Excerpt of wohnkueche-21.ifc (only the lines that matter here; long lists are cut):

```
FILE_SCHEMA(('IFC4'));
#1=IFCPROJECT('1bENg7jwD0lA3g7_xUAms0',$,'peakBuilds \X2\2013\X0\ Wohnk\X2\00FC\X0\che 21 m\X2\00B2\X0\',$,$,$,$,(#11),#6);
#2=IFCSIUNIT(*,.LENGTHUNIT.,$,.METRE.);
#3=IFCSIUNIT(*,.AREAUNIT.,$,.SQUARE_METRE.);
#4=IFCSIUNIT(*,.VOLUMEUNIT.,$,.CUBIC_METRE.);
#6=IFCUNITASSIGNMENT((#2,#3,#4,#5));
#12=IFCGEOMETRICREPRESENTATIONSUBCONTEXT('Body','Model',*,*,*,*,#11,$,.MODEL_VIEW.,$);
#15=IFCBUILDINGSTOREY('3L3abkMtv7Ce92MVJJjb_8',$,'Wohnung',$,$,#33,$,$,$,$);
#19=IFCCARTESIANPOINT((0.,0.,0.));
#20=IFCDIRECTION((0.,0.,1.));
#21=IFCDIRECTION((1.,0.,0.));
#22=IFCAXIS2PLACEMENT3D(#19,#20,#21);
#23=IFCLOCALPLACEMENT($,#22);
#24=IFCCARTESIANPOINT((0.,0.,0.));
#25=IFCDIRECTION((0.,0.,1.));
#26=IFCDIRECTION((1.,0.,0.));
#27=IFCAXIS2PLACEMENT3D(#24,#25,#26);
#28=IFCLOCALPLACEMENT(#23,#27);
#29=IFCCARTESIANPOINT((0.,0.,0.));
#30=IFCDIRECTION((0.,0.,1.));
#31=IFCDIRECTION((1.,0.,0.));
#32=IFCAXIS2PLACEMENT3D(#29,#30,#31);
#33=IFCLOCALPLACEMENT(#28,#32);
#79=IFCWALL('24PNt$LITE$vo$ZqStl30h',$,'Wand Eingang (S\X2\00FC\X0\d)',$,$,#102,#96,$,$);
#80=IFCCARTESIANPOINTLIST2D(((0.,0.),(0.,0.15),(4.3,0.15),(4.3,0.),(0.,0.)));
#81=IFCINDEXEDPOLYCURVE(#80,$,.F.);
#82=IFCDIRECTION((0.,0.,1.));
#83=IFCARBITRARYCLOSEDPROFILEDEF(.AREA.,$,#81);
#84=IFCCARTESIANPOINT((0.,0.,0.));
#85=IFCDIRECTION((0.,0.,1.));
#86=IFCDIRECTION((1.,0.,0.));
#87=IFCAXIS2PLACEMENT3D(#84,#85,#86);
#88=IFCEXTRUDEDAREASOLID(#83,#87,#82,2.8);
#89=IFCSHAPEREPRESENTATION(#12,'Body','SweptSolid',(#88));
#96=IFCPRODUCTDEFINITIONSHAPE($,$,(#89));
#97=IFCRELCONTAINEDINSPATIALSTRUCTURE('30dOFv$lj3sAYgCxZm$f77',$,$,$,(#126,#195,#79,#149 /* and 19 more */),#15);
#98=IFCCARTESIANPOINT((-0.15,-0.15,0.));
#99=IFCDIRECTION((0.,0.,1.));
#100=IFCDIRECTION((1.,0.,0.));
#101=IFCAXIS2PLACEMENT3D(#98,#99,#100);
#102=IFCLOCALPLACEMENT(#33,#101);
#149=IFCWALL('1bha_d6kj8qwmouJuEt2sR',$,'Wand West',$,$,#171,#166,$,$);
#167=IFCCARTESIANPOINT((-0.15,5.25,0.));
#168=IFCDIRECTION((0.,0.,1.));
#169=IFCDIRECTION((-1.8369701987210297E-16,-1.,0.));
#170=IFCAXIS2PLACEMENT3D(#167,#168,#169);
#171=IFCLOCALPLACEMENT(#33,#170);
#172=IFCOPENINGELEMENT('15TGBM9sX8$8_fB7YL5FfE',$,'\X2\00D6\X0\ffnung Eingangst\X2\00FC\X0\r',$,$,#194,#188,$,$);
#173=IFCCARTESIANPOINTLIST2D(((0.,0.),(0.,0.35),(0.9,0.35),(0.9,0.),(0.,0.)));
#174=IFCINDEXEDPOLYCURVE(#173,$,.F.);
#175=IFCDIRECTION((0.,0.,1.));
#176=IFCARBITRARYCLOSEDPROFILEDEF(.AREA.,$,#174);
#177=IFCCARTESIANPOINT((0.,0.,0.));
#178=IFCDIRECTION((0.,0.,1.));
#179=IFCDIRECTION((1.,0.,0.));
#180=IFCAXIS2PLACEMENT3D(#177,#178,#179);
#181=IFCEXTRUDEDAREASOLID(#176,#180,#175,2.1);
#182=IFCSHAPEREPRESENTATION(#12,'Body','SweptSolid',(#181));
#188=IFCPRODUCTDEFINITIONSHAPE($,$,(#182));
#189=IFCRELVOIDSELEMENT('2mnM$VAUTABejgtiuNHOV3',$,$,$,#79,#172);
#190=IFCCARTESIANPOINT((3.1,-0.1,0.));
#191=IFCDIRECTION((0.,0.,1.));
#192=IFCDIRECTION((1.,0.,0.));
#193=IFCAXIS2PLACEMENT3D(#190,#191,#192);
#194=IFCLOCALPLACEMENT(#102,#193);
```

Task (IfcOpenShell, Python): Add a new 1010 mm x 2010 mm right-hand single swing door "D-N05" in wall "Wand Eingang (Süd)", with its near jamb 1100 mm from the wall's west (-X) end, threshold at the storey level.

```python
import numpy as np
import ifcopenshell
import ifcopenshell.api.feature
import ifcopenshell.api.geometry
import ifcopenshell.api.root
import ifcopenshell.api.spatial
import ifcopenshell.geom
import ifcopenshell.util.element
import ifcopenshell.util.placement
import ifcopenshell.util.representation
import ifcopenshell.util.shape
import ifcopenshell.util.unit

model = ifcopenshell.open("wohnkueche-21.ifc")
unit_scale = ifcopenshell.util.unit.calculate_unit_scale(model)
settings = ifcopenshell.geom.settings()


def volume(element):
    """Net volume in cubic metres, openings subtracted."""
    shape = ifcopenshell.geom.create_shape(settings, element)
    return ifcopenshell.util.shape.get_volume(shape.geometry)


wall = model.by_id(79)
storey = ifcopenshell.util.element.get_container(wall, ifc_class="IfcBuildingStorey")
context = ifcopenshell.util.representation.get_context(model, "Model", "Body", "MODEL_VIEW")
before = volume(wall)

width, height, from_end, sill = 1.01, 2.01, 1.1, 0.0  # metres

# The wall runs along its own X axis, and the end named is its -X end.
wall_shape = ifcopenshell.geom.create_shape(settings, wall)
x, y, z = ifcopenshell.util.shape.get_vertices(wall_shape.geometry).T
start = x.min() + from_end
face, thickness = float(y.min()), float(y.max() - y.min())
wall_matrix = ifcopenshell.util.placement.get_local_placement(wall.ObjectPlacement)
level = ifcopenshell.util.placement.get_local_placement(storey.ObjectPlacement)[2, 3]


def in_wall(x, y):
    """Placement at x, y metres in the wall's axes, at sill height."""
    matrix = wall_matrix.copy()
    matrix[:, 3] = wall_matrix @ np.array([x / unit_scale, y / unit_scale, 0.0, 1.0])
    matrix[2, 3] = level + sill / unit_scale
    return matrix


# Opening: a box that overshoots both wall faces by 50 mm.
opening = ifcopenshell.api.root.create_entity(model, ifc_class="IfcOpeningElement", predefined_type="OPENING")
box = ifcopenshell.api.geometry.add_wall_representation(
    model, context=context, length=width, height=height, thickness=thickness + 0.1
)
ifcopenshell.api.geometry.assign_representation(model, product=opening, representation=box)
ifcopenshell.api.geometry.edit_object_placement(model, product=opening, matrix=in_wall(start, face - 0.05), is_si=False)
ifcopenshell.api.feature.add_feature(model, feature=opening, element=wall)

door = ifcopenshell.api.root.create_entity(model, ifc_class="IfcDoor", name="D-N05", predefined_type="DOOR")
door.OverallWidth, door.OverallHeight = width / unit_scale, height / unit_scale
door.OperationType = "SINGLE_SWING_RIGHT"
body = ifcopenshell.api.geometry.add_door_representation(
    model,
    context=context,
    overall_width=door.OverallWidth,
    overall_height=door.OverallHeight,
    operation_type="SINGLE_SWING_RIGHT",
    lining_properties={"LiningDepth": thickness / unit_scale, "ThresholdDepth": thickness / unit_scale},
)
ifcopenshell.api.geometry.assign_representation(model, product=door, representation=body)
ifcopenshell.api.spatial.assign_container(model, products=[door], relating_structure=storey)
ifcopenshell.api.feature.add_filling(model, opening=opening, element=door)

# The lining spans the wall, so the door starts at the wall face.
ifcopenshell.api.geometry.edit_object_placement(model, product=door, matrix=in_wall(start, face), is_si=False)

after = volume(wall)

print(f"wall volume {before:.3f} -> {after:.3f} m3")

model.write("wohnkueche-21-out.ifc")
```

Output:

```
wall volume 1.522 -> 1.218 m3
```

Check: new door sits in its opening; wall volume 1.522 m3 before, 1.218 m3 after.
